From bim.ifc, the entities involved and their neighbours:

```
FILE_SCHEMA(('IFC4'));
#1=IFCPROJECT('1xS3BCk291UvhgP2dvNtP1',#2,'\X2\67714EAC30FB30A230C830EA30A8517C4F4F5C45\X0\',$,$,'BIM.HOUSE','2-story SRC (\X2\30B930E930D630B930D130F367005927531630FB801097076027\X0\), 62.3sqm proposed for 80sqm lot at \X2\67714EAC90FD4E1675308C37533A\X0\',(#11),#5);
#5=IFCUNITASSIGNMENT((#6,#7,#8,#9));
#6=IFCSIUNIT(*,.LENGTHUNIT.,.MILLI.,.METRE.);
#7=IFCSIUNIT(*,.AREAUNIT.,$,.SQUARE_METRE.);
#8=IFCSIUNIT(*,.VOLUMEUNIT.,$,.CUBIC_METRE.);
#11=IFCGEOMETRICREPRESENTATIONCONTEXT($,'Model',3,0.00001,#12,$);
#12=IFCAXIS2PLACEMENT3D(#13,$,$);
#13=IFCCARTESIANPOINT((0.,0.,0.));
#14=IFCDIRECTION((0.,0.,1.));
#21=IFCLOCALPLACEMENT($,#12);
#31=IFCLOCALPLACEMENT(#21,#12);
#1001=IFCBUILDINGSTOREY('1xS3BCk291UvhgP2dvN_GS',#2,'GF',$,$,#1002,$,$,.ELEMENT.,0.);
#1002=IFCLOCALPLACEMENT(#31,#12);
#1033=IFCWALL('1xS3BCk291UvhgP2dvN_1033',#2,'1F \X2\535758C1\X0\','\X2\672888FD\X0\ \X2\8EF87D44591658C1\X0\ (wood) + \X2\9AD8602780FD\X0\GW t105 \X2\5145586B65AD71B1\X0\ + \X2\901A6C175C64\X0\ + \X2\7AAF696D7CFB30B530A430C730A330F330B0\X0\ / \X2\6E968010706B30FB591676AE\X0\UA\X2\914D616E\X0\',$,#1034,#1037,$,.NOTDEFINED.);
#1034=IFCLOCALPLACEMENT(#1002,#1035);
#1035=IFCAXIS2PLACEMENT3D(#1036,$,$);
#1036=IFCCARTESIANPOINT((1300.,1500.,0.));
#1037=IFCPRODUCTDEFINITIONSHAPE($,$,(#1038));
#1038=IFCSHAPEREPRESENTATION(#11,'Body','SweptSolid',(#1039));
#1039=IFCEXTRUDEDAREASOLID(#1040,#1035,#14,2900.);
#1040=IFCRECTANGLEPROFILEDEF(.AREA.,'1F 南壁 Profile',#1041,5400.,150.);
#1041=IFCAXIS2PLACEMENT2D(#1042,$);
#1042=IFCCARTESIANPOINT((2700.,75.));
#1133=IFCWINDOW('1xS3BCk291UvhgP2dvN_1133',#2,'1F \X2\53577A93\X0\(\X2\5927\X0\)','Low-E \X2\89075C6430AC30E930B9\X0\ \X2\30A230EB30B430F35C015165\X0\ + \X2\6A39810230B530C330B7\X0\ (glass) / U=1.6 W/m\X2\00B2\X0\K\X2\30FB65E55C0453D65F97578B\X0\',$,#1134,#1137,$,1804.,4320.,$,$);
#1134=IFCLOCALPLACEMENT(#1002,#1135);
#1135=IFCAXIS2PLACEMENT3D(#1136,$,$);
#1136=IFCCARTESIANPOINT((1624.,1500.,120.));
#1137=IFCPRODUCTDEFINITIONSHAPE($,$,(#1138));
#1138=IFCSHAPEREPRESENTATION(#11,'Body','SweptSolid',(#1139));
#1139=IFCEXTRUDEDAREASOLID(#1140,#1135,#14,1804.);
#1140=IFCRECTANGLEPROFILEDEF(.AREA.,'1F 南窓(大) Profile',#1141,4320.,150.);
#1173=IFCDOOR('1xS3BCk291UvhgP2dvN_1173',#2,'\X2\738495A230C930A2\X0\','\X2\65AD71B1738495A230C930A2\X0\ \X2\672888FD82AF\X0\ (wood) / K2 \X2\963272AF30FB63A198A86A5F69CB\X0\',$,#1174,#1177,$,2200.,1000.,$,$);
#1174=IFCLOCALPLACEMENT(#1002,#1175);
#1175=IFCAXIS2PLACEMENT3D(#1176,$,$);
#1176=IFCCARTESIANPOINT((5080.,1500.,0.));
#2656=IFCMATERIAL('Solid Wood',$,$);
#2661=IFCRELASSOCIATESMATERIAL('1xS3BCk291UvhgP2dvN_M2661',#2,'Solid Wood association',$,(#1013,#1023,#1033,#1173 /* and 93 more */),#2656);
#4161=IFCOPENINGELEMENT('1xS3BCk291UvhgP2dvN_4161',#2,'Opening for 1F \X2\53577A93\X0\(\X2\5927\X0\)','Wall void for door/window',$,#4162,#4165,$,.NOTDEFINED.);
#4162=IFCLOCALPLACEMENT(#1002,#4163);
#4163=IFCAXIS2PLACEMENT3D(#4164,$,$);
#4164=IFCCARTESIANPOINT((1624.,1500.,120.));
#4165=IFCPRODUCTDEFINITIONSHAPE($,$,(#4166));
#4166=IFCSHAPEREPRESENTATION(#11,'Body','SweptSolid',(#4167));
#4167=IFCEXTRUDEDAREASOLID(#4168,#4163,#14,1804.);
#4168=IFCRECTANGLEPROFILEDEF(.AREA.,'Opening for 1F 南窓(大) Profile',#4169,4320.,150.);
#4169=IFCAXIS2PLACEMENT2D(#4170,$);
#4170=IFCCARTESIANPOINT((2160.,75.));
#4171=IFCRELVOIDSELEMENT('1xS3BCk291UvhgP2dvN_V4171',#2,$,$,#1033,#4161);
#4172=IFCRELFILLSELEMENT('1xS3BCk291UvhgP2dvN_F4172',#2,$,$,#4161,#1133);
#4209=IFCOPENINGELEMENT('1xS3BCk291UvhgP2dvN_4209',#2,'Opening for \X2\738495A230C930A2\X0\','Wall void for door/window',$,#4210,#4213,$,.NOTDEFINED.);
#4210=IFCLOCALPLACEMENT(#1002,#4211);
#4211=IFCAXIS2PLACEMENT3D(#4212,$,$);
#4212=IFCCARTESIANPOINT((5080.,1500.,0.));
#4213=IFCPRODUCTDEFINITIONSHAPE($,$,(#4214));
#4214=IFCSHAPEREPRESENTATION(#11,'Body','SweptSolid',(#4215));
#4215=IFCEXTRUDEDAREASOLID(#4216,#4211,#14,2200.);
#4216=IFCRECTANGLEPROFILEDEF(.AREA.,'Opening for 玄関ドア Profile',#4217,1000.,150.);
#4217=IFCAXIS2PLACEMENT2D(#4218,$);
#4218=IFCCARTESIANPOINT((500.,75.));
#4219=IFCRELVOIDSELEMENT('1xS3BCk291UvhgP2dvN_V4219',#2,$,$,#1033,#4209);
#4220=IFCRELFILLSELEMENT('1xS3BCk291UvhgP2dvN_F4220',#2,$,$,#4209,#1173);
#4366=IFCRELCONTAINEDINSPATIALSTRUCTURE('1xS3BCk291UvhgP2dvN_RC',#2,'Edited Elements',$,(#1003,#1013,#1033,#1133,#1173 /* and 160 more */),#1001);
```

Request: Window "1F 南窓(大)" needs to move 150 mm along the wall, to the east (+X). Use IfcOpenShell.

```python
import ifcopenshell
import ifcopenshell.api.geometry
import ifcopenshell.util.placement

model = ifcopenshell.open("bim.ifc")

window = model.by_guid("1xS3BCk291UvhgP2dvN_1133")
opening = window.FillsVoids[0].RelatingOpeningElement
wall = opening.VoidsElements[0].RelatingBuildingElement

wall_matrix = ifcopenshell.util.placement.get_local_placement(wall.ObjectPlacement)
shift = wall_matrix[:3, 0] * 150.0
before = ifcopenshell.util.placement.get_local_placement(window.ObjectPlacement)[:3, 3].copy()

# The window is not placed relative to its opening, so move both.
for product in (opening, window):
    matrix = ifcopenshell.util.placement.get_local_placement(product.ObjectPlacement)
    matrix[:3, 3] += shift
    ifcopenshell.api.geometry.edit_object_placement(model, product=product, matrix=matrix, is_si=False)

after = ifcopenshell.util.placement.get_local_placement(window.ObjectPlacement)[:3, 3]
print("window moved by", (after - before).round(3) + 0.0)

model.write("bim_v2.ifc")
```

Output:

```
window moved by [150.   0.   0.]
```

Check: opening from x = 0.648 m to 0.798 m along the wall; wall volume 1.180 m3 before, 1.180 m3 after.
